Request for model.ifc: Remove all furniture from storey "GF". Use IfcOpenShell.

First a look at what the model holds.

```python
import ifcopenshell
import ifcopenshell.util.element

model = ifcopenshell.open("model.ifc")
print(model.schema)
storey = next(s for s in model.by_type("IfcBuildingStorey") if s.Name == "GF")
furniture = [e for e in ifcopenshell.util.element.get_decomposition(storey) if e.is_a("IfcFurnishingElement")]
seen = {}
for e in furniture:
    element_type = ifcopenshell.util.element.get_type(e)
    name = element_type.Name if element_type not in (None, e) else None
    seen[name] = seen.get(name, 0) + 1
for name, count in sorted(seen.items(), key=str):
    print(count, "x", name)
```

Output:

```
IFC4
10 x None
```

```python
import ifcopenshell
import ifcopenshell.api.root
import ifcopenshell.util.element

model = ifcopenshell.open("model.ifc")

storey = next(s for s in model.by_type("IfcBuildingStorey") if s.Name == "GF")
furniture = [e for e in ifcopenshell.util.element.get_decomposition(storey) if e.is_a("IfcFurnishingElement")]

for e in furniture:
    ifcopenshell.api.root.remove_product(model, product=e)
print(len(furniture), "removed")

model.write("model_v2.ifc")
```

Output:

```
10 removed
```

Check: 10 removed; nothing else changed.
